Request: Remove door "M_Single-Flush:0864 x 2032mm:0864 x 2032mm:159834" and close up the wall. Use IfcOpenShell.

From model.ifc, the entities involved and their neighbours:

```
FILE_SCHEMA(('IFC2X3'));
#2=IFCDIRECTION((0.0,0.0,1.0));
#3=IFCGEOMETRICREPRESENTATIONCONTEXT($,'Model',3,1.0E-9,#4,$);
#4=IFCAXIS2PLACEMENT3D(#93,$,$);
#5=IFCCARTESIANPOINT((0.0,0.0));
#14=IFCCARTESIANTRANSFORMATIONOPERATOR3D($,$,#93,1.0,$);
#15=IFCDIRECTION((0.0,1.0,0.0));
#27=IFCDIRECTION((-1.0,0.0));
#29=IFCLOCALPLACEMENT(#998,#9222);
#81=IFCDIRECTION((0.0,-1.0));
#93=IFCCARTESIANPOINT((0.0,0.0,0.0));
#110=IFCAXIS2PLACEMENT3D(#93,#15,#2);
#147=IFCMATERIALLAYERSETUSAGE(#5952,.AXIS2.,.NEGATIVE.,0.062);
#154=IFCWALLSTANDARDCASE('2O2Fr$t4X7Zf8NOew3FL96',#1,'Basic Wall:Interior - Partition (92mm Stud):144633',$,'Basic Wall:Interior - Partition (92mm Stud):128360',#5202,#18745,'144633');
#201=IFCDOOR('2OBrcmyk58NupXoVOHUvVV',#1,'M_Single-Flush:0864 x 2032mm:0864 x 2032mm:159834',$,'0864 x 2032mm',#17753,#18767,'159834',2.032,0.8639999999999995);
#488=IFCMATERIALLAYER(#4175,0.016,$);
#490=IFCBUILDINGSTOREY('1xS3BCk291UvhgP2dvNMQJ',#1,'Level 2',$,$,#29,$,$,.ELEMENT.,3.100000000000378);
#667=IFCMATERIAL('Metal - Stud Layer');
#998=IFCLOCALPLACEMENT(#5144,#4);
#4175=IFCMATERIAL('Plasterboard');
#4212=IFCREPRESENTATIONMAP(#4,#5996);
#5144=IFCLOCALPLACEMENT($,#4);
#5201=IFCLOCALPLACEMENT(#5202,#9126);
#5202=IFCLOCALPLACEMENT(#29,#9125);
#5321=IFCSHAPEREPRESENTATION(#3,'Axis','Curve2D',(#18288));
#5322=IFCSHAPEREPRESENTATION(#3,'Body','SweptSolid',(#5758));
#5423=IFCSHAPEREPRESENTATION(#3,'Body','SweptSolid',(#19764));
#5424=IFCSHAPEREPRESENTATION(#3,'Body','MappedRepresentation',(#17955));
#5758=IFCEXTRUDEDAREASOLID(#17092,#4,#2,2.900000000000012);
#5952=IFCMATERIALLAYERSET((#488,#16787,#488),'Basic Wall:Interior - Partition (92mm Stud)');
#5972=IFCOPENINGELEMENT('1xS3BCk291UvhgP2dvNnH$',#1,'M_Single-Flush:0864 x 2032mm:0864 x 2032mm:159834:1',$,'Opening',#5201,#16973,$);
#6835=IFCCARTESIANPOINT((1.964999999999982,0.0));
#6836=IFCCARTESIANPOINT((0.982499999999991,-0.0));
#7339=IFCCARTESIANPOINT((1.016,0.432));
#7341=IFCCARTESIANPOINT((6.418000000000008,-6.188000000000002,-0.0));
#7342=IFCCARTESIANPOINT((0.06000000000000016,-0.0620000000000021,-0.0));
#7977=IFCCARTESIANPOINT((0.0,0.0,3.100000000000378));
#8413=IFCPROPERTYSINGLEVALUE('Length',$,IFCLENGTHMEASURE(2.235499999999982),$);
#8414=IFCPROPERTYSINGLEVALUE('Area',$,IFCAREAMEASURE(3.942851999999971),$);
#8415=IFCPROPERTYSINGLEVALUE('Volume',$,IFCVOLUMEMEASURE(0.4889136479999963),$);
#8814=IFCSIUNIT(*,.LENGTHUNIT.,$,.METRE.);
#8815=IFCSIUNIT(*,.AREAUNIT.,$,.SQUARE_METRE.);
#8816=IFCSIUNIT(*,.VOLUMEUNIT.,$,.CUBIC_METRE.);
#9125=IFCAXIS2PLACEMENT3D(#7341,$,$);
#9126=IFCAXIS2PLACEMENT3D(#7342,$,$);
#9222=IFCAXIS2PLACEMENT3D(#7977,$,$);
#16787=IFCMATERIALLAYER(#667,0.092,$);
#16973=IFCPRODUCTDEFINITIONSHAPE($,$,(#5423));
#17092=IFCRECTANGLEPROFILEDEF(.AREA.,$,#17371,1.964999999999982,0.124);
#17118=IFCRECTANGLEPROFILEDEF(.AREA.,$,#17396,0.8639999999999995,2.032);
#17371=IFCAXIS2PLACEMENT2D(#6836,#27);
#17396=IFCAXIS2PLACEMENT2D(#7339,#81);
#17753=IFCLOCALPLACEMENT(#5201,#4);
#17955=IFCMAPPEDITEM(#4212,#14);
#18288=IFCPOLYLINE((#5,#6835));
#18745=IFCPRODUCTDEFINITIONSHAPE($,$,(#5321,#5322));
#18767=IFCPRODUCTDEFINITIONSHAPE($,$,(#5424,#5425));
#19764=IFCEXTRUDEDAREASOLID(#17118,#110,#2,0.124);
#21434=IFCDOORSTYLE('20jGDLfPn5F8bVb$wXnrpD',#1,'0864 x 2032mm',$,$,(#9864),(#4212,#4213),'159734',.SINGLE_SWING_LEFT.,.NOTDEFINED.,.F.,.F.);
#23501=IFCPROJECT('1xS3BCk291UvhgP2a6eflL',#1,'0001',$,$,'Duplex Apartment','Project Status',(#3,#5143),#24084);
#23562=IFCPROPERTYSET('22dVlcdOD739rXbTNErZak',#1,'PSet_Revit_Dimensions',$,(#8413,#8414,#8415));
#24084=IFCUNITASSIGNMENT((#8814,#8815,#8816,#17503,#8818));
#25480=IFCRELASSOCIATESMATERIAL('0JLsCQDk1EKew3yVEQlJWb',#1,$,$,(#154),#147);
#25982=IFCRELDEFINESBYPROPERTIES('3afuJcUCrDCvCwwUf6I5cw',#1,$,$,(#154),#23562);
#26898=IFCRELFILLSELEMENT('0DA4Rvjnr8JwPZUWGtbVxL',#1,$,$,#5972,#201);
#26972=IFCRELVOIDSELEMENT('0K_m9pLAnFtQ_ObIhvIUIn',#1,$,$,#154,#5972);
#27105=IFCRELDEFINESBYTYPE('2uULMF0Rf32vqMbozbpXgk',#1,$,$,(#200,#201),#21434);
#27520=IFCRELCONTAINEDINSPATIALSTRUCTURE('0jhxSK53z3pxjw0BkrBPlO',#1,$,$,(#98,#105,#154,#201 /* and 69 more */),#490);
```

```python
import ifcopenshell
import ifcopenshell.api.feature
import ifcopenshell.api.pset
import ifcopenshell.api.root
import ifcopenshell.geom
import ifcopenshell.util.element
import ifcopenshell.util.shape
import ifcopenshell.util.unit

model = ifcopenshell.open("model.ifc")
area_scale = ifcopenshell.util.unit.calculate_unit_scale(model, "AREAUNIT")
volume_scale = ifcopenshell.util.unit.calculate_unit_scale(model, "VOLUMEUNIT")
settings = ifcopenshell.geom.settings()


def volume(element):
    """Net volume in cubic metres, openings subtracted."""
    shape = ifcopenshell.geom.create_shape(settings, element)
    return ifcopenshell.util.shape.get_volume(shape.geometry)


door = model.by_id(201)
opening = door.FillsVoids[0].RelatingOpeningElement
wall = opening.VoidsElements[0].RelatingBuildingElement
before = volume(wall)

ifcopenshell.api.root.remove_product(model, product=door)
ifcopenshell.api.feature.remove_feature(model, feature=opening)

after = volume(wall)
thickness = 0.124  # wall thickness in metres

# Update the wall's stored quantities.
pset = model.by_id(ifcopenshell.util.element.get_pset(wall, "PSet_Revit_Dimensions", should_inherit=False)["id"])
ifcopenshell.api.pset.edit_pset(model, pset=pset, properties={
    "Area": model.create_entity("IfcAreaMeasure", after / thickness / area_scale),
    "Volume": model.create_entity("IfcVolumeMeasure", after / volume_scale),
})

print(f"wall volume {before:.3f} -> {after:.3f} m3")

model.write("model_edited.ifc")
```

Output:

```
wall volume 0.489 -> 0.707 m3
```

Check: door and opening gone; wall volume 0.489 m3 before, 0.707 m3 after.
